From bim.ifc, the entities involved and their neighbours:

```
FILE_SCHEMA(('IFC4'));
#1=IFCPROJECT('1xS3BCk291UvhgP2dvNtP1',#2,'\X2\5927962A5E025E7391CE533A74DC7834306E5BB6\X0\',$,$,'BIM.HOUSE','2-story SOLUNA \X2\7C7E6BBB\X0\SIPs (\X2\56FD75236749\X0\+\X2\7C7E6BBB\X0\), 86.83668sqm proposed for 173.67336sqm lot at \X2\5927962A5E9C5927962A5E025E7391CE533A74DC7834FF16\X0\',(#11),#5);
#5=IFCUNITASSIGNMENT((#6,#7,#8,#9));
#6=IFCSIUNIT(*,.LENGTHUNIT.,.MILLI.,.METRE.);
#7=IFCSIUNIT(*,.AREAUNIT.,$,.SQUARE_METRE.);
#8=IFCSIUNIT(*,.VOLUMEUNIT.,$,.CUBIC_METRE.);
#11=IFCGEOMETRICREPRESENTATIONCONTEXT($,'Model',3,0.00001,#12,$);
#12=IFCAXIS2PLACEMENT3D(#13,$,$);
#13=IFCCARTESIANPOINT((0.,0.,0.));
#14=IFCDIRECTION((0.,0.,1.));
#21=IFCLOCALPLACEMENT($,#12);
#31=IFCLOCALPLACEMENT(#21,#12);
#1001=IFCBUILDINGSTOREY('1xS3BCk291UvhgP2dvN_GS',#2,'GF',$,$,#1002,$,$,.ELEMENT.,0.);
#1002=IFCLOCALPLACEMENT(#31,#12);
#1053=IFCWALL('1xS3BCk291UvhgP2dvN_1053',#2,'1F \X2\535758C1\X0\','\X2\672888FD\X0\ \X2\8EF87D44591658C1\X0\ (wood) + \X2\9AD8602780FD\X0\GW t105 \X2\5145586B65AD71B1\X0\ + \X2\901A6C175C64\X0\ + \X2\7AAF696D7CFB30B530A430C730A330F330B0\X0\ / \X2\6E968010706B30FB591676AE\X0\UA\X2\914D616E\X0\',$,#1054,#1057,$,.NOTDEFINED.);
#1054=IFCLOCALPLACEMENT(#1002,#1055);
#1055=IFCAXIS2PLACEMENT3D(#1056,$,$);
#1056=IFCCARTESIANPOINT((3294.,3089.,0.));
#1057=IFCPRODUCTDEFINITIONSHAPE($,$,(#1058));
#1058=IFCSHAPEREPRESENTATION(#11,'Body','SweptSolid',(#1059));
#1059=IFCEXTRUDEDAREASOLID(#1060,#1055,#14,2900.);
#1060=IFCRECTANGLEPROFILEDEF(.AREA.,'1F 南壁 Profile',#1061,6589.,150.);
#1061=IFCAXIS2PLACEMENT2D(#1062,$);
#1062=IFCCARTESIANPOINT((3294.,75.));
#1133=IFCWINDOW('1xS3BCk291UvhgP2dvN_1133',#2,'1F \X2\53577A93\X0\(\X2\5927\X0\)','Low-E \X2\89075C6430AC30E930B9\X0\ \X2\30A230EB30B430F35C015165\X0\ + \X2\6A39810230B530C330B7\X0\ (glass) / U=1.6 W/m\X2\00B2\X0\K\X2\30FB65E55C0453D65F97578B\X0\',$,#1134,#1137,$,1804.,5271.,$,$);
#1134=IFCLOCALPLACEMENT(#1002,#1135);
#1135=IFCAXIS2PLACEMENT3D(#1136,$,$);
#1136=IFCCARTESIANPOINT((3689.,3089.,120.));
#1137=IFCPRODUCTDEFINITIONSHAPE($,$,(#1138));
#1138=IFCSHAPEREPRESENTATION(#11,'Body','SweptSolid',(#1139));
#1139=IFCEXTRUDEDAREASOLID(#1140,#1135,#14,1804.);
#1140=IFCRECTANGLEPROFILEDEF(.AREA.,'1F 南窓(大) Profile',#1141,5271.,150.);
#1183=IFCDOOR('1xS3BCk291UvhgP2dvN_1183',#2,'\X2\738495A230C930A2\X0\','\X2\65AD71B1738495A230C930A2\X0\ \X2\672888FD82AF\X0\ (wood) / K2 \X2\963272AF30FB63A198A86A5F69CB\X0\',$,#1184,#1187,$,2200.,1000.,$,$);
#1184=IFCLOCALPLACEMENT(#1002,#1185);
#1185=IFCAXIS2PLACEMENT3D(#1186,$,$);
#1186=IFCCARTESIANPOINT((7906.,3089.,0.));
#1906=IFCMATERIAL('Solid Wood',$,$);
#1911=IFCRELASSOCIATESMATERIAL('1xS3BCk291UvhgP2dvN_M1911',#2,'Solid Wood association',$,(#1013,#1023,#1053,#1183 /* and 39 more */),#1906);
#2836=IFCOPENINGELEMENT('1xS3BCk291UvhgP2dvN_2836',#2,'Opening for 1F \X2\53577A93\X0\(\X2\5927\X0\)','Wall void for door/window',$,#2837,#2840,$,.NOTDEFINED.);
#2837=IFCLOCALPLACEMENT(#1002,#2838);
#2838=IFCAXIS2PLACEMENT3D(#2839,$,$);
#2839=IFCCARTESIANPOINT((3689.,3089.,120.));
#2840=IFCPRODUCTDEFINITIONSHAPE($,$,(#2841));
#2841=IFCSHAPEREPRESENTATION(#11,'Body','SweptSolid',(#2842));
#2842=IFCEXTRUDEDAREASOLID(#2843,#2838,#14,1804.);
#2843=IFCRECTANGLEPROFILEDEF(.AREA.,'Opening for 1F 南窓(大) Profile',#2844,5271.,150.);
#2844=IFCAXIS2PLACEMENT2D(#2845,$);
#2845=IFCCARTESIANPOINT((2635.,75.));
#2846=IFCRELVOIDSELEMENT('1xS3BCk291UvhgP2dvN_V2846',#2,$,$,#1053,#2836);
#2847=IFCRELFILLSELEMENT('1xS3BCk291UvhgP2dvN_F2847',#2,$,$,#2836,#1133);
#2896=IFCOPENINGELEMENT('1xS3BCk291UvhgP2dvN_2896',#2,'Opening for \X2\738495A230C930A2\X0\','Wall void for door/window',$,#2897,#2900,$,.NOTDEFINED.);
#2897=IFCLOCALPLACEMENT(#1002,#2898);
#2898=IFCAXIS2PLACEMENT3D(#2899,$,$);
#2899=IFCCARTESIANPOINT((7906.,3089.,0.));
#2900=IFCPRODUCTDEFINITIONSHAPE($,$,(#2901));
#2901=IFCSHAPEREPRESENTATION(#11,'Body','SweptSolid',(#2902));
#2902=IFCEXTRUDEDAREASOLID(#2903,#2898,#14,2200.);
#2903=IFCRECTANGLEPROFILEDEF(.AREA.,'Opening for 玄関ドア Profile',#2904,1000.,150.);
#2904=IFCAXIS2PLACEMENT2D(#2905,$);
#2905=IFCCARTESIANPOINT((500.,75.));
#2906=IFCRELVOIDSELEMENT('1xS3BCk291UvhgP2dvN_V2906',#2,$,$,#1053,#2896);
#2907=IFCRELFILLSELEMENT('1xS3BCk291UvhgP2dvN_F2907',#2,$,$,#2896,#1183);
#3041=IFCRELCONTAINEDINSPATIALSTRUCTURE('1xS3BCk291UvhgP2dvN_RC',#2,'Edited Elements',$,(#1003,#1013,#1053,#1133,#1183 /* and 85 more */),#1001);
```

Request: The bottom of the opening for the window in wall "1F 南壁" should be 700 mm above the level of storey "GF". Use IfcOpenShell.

```python
import numpy as np
import ifcopenshell
import ifcopenshell.api.geometry
import ifcopenshell.geom
import ifcopenshell.util.element
import ifcopenshell.util.placement
import ifcopenshell.util.shape
import ifcopenshell.util.unit

model = ifcopenshell.open("bim.ifc")
unit_scale = ifcopenshell.util.unit.calculate_unit_scale(model)

window = model.by_guid("1xS3BCk291UvhgP2dvN_1133")
opening = window.FillsVoids[0].RelatingOpeningElement
storey = ifcopenshell.util.element.get_container(window, ifc_class="IfcBuildingStorey")
level = ifcopenshell.util.placement.get_local_placement(storey.ObjectPlacement)[2, 3]

# The opening's origin need not be at the sill, so measure its lowest point.
shape = ifcopenshell.geom.create_shape(ifcopenshell.geom.settings(), opening)
bottom = ifcopenshell.util.shape.get_shape_bottom_elevation(shape, shape.geometry) / unit_scale
dz = level + 0.7 / unit_scale - bottom

shift = np.array([0.0, 0.0, dz])
# The window is not placed relative to its opening, so move both.
for product in (opening, window):
    matrix = ifcopenshell.util.placement.get_local_placement(product.ObjectPlacement)
    matrix[:3, 3] += shift
    ifcopenshell.api.geometry.edit_object_placement(model, product=product, matrix=matrix, is_si=False)

print(f"moved by {dz * unit_scale:+.3f} m")

model.write("bim-out.ifc")
```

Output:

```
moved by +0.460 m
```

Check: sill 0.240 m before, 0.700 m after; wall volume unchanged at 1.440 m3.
